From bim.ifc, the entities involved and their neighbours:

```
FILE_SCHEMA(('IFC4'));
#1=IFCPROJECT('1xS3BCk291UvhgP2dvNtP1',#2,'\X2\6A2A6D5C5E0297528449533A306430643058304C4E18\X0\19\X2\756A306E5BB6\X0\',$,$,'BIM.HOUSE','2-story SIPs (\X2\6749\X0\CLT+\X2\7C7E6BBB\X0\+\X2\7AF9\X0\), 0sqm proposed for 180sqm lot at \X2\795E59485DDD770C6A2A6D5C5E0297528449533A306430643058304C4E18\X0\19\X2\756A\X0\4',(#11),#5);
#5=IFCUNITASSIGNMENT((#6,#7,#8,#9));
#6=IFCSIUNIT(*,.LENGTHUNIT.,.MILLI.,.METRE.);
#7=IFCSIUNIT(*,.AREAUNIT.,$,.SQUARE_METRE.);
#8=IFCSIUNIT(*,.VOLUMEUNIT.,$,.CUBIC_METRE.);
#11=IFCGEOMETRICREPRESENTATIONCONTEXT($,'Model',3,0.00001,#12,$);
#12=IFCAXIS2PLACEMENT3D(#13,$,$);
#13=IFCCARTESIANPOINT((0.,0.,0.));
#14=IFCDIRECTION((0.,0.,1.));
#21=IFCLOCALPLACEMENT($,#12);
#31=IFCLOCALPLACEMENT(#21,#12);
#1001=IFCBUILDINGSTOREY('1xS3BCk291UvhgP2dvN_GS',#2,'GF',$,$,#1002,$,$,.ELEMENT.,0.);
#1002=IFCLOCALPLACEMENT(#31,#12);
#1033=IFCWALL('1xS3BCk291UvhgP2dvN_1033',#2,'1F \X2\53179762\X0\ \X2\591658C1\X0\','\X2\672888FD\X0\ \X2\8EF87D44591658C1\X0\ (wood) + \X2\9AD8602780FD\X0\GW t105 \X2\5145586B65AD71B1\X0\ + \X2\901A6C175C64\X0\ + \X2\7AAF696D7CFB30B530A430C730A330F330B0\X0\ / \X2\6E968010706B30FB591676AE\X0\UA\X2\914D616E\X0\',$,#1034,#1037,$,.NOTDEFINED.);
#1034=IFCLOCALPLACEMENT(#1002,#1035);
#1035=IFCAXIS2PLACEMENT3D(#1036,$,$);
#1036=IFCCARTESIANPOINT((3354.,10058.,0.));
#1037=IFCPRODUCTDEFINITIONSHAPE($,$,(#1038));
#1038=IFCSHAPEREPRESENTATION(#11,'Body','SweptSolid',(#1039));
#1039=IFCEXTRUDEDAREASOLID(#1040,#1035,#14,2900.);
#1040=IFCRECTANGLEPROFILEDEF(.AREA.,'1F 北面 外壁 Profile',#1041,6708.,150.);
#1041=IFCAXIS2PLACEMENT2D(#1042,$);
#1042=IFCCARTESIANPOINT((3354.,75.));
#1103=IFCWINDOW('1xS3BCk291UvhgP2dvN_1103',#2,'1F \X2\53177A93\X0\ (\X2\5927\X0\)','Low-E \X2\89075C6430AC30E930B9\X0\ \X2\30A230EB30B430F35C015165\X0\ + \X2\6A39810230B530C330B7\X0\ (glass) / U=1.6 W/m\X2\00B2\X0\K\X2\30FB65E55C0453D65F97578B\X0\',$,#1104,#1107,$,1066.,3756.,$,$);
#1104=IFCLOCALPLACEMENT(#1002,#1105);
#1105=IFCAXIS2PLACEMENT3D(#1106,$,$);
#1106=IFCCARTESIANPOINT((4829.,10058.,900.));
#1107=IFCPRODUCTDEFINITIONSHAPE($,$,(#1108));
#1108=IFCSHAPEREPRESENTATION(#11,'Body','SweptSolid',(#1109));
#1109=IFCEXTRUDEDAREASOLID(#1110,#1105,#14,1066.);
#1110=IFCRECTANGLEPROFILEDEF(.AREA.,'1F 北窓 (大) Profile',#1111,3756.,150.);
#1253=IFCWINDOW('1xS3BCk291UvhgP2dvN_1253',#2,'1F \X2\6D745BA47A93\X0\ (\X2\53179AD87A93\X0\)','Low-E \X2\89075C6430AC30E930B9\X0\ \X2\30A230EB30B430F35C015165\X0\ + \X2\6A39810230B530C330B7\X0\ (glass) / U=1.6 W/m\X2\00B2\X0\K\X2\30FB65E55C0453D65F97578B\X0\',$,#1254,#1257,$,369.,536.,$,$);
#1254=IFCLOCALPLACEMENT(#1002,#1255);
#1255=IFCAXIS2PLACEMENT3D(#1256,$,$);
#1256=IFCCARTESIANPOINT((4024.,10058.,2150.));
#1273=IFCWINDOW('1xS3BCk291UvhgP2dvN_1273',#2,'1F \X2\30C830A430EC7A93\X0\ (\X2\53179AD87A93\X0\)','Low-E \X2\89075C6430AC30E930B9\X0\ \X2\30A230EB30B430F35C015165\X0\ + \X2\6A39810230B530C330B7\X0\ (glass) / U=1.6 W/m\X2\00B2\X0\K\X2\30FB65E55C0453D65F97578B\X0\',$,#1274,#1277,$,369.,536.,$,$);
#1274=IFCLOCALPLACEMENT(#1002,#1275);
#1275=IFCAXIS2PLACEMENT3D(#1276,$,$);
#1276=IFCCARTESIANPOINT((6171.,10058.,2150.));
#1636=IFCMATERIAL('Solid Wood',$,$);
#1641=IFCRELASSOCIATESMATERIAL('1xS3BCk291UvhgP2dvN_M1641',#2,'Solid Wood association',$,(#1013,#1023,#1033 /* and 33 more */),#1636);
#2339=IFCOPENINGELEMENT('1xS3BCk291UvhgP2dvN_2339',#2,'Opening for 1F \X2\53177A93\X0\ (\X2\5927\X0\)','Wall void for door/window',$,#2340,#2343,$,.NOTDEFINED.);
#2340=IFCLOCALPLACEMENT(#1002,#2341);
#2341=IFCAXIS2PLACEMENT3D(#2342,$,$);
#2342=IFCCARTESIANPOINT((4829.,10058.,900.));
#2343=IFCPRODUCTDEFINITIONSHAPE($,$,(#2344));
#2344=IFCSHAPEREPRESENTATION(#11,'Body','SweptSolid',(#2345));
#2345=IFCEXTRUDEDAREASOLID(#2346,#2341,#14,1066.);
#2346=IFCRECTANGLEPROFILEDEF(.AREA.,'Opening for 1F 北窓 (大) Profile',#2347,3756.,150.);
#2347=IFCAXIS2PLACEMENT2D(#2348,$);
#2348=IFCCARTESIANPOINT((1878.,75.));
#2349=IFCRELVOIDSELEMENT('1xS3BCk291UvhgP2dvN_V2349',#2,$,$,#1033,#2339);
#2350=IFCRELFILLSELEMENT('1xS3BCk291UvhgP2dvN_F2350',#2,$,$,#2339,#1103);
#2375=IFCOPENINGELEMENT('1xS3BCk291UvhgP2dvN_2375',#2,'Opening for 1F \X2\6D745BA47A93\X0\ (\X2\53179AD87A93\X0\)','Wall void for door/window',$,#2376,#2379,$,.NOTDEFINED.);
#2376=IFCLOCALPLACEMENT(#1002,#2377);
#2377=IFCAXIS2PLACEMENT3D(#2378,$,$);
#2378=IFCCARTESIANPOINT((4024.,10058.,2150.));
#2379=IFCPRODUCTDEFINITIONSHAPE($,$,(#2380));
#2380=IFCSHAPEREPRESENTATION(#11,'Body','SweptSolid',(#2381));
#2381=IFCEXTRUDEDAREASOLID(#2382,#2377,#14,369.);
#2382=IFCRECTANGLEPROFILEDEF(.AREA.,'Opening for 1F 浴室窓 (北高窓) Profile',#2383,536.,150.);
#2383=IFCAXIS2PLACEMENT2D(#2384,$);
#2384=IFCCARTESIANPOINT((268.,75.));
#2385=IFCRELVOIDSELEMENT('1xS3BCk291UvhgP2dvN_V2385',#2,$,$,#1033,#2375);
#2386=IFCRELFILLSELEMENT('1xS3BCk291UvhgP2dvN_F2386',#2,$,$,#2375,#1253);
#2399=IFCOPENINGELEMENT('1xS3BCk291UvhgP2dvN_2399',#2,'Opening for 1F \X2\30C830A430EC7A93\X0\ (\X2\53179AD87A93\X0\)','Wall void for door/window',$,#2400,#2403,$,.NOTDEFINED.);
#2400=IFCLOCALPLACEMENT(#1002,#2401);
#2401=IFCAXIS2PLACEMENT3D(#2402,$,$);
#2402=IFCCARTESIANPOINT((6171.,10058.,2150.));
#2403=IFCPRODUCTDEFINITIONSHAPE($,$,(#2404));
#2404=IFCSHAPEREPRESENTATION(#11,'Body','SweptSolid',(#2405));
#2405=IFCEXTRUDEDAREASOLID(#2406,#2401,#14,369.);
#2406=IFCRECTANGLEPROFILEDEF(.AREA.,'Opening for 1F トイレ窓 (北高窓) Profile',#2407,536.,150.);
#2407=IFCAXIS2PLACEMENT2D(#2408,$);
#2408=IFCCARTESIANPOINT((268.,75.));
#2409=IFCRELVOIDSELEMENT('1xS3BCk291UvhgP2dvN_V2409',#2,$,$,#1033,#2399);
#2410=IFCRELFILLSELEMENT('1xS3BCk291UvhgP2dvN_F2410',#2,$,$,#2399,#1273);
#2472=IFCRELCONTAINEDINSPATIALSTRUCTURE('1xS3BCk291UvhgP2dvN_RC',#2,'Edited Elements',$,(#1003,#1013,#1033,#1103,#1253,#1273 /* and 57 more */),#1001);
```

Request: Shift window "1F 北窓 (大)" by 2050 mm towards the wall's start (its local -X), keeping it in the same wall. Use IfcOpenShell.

```python
import ifcopenshell
import ifcopenshell.api.geometry
import ifcopenshell.util.placement

model = ifcopenshell.open("bim.ifc")

window = model.by_guid("1xS3BCk291UvhgP2dvN_1103")
opening = window.FillsVoids[0].RelatingOpeningElement
wall = opening.VoidsElements[0].RelatingBuildingElement

wall_matrix = ifcopenshell.util.placement.get_local_placement(wall.ObjectPlacement)
shift = wall_matrix[:3, 0] * -2050.0
before = ifcopenshell.util.placement.get_local_placement(window.ObjectPlacement)[:3, 3].copy()

# The window is not placed relative to its opening, so move both.
for product in (opening, window):
    matrix = ifcopenshell.util.placement.get_local_placement(product.ObjectPlacement)
    matrix[:3, 3] += shift
    ifcopenshell.api.geometry.edit_object_placement(model, product=product, matrix=matrix, is_si=False)

after = ifcopenshell.util.placement.get_local_placement(window.ObjectPlacement)[:3, 3]
print("window moved by", (after - before).round(3) + 0.0)

model.write("bim_rev.ifc")
```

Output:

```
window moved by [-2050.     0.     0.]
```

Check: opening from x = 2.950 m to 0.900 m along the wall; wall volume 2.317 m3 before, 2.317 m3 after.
